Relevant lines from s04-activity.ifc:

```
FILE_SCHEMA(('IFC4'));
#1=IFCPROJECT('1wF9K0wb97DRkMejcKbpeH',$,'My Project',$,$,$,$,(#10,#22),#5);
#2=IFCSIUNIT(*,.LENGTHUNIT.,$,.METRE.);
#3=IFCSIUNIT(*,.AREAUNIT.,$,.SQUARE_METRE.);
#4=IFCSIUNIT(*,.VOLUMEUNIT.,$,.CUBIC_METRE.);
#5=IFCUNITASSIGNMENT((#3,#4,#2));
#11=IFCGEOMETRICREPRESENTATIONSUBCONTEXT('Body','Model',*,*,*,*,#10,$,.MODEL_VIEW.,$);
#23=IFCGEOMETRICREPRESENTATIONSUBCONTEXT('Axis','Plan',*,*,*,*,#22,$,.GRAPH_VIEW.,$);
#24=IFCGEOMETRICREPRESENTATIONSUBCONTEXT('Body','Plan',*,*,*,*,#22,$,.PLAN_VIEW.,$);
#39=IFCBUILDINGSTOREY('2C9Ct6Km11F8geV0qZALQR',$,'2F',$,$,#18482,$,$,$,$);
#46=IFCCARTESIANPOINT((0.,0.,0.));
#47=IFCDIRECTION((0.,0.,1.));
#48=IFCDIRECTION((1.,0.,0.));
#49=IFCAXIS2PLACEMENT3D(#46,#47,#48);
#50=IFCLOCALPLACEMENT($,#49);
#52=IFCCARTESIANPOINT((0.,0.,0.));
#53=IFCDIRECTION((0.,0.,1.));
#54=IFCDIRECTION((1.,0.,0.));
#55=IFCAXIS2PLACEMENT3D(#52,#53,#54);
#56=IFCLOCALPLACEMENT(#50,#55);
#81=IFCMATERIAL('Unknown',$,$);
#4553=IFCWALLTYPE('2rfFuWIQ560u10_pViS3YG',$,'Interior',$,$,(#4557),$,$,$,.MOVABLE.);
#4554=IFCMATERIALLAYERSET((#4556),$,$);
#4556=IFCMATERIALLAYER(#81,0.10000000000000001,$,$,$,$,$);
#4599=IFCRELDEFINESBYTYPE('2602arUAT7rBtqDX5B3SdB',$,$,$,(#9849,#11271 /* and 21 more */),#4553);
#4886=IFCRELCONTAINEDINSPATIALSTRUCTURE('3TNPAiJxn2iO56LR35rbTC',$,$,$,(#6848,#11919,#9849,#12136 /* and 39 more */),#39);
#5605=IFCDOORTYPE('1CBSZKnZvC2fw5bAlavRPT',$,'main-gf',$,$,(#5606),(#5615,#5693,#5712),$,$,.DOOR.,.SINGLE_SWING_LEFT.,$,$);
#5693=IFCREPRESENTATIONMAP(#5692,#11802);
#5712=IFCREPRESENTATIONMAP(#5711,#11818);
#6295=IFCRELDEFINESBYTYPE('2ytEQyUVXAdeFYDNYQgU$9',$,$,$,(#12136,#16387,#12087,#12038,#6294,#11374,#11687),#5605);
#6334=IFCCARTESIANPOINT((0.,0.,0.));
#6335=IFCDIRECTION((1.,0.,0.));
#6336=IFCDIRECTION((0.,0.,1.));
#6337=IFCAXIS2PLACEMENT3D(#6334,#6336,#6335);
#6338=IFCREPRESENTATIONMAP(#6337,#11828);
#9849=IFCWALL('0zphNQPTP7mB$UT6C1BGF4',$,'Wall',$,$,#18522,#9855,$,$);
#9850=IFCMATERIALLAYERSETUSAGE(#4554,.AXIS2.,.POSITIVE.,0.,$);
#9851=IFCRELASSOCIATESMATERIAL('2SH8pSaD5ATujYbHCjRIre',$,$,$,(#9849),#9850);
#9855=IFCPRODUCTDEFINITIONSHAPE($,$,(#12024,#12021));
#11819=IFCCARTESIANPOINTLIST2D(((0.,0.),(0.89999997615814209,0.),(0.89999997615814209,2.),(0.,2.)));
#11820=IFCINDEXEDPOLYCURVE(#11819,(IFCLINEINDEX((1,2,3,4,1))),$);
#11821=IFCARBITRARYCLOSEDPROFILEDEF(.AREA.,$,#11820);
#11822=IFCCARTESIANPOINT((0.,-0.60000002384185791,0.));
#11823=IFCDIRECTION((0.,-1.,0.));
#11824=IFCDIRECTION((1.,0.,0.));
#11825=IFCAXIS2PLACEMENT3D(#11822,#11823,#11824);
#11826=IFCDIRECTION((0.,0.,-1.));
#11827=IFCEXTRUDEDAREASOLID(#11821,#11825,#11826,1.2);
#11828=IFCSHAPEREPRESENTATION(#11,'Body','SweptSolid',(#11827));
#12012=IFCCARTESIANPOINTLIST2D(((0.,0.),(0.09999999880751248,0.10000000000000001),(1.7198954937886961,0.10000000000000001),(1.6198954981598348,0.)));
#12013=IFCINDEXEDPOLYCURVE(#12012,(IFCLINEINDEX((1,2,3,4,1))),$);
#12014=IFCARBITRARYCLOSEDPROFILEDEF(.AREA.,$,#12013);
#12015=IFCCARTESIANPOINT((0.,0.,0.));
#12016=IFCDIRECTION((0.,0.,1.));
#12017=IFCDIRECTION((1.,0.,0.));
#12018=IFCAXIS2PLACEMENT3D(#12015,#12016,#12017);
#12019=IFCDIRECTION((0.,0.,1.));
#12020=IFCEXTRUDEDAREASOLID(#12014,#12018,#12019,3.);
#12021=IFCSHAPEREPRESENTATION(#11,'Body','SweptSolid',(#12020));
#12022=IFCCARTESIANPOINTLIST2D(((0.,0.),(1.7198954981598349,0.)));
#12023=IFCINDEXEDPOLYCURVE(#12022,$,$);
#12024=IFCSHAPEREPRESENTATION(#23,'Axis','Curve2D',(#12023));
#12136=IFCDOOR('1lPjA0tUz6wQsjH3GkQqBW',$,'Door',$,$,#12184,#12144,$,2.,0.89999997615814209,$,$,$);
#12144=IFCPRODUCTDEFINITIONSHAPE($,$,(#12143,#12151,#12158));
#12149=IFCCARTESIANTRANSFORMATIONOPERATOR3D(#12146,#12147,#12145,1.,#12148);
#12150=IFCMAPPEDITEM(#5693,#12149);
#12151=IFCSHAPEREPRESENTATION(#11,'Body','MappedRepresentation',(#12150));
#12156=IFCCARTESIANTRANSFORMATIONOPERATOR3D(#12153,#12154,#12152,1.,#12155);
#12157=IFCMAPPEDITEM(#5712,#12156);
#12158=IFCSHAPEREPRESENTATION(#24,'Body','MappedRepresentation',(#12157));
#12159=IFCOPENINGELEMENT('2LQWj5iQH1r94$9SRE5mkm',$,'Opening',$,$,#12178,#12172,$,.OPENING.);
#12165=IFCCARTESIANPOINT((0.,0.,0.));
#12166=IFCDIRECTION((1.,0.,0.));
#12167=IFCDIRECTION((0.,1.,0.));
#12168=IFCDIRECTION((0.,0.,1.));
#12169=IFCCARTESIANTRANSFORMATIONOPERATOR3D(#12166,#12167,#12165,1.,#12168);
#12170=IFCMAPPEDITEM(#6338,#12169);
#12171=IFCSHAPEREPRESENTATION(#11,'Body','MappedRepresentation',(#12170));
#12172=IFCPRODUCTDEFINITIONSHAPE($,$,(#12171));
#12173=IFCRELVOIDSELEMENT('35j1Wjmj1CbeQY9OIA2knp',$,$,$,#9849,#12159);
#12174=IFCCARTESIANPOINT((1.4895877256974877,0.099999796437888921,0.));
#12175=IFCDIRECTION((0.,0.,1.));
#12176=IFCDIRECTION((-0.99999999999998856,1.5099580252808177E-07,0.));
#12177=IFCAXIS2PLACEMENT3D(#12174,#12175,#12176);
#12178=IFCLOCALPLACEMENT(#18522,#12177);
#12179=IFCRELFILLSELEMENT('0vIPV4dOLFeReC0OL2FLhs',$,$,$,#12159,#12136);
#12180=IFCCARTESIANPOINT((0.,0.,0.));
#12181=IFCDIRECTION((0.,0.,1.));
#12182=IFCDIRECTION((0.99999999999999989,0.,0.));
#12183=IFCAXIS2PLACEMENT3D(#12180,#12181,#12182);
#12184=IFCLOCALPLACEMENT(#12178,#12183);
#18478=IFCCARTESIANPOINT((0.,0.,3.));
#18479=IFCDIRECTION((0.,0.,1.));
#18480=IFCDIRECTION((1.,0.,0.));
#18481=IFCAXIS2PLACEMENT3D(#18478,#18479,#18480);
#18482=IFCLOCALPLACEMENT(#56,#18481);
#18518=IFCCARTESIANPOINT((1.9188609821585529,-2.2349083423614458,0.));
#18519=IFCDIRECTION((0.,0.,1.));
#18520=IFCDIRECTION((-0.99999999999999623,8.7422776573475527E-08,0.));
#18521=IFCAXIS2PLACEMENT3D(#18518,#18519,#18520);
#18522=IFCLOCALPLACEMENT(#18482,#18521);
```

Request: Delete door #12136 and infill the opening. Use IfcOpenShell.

```python
import ifcopenshell
import ifcopenshell.api.feature
import ifcopenshell.api.root
import ifcopenshell.geom
import ifcopenshell.util.shape

model = ifcopenshell.open("s04-activity.ifc")
settings = ifcopenshell.geom.settings()


def volume(element):
    """Net volume in cubic metres, openings subtracted."""
    shape = ifcopenshell.geom.create_shape(settings, element)
    return ifcopenshell.util.shape.get_volume(shape.geometry)


door = model.by_guid("1lPjA0tUz6wQsjH3GkQqBW")
opening = door.FillsVoids[0].RelatingOpeningElement
wall = opening.VoidsElements[0].RelatingBuildingElement
before = volume(wall)

ifcopenshell.api.root.remove_product(model, product=door)
ifcopenshell.api.feature.remove_feature(model, feature=opening)

after = volume(wall)

print(f"wall volume {before:.3f} -> {after:.3f} m3")

model.write("s04-activity_v2.ifc")
```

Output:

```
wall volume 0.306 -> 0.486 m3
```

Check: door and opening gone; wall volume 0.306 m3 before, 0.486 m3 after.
